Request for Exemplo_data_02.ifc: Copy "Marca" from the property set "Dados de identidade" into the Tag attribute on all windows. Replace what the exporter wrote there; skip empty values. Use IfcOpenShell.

First a look at what the model holds.

```python
import ifcopenshell
import ifcopenshell.util.element

model = ifcopenshell.open("Exemplo_data_02.ifc")
print(model.schema)
windows = model.by_type("IfcWindow")
print(len(windows), "windows")
for e in windows[:8]:
    source = ifcopenshell.util.element.get_pset(e, "Dados de identidade", "Marca")
    target = e.Tag
    print(e.id(), repr(source), repr(target), sep=" | ")
```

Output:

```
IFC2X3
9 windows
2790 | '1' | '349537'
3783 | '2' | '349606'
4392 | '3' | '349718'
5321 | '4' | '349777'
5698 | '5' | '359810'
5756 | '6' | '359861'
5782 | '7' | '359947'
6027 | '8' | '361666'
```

```python
import ifcopenshell
import ifcopenshell.util.element

model = ifcopenshell.open("Exemplo_data_02.ifc")

count = 0
for e in model.by_type("IfcWindow"):
    value = ifcopenshell.util.element.get_pset(e, "Dados de identidade", "Marca")
    current = e.Tag
    if not value or not value.strip() or current == value:
        continue
    e.Tag = value
    count += 1

print(count, "windows updated")

model.write("Exemplo_data_02_v2.ifc")
```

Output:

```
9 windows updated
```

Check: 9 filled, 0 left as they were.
